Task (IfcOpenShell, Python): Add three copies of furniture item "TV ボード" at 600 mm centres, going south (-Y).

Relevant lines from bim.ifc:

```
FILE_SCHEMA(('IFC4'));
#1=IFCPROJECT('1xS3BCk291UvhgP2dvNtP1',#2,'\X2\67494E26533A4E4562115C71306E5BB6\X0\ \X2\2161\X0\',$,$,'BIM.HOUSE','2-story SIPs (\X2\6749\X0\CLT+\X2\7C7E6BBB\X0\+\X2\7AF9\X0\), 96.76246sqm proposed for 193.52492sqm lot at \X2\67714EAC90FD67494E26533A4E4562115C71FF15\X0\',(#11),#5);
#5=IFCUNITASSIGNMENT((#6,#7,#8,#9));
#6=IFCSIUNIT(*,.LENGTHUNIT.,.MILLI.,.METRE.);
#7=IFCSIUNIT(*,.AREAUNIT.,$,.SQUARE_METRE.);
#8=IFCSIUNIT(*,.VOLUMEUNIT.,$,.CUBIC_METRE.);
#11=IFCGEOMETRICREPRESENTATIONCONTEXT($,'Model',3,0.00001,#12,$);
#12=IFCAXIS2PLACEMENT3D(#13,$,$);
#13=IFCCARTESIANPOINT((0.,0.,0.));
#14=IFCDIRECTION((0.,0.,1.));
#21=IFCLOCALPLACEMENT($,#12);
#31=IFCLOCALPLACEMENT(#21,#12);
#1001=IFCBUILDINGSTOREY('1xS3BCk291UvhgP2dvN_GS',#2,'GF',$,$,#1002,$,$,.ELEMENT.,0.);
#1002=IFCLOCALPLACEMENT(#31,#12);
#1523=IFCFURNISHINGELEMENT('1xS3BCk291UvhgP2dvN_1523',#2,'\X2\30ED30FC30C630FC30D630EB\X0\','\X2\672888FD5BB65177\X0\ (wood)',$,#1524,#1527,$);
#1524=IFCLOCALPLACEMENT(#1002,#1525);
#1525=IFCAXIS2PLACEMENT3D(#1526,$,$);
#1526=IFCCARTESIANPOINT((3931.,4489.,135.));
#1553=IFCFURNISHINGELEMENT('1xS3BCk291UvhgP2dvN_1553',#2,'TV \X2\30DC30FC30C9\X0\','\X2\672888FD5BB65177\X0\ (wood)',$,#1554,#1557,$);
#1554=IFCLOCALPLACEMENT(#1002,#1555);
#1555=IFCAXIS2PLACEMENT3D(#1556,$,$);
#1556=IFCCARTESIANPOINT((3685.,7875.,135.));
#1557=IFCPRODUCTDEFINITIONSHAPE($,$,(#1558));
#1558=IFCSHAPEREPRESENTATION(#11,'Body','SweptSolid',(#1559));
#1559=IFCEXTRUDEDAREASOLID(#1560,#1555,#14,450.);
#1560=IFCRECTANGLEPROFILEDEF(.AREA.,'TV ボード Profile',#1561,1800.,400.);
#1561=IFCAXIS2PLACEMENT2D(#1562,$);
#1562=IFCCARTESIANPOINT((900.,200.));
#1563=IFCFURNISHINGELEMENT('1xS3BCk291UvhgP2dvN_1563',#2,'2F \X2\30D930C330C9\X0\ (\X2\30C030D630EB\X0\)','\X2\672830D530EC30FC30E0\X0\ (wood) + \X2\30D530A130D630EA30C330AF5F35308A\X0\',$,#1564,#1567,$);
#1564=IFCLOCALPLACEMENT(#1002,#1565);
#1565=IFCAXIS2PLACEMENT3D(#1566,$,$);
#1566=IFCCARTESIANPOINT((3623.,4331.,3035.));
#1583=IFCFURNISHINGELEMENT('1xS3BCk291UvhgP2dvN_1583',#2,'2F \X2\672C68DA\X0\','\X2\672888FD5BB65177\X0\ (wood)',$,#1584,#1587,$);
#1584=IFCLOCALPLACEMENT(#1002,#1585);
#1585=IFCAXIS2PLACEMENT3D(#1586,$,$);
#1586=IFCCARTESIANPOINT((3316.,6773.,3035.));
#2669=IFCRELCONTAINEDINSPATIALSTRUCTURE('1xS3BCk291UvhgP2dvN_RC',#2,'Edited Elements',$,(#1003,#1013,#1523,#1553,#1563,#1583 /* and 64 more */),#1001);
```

```python
import numpy as np
import ifcopenshell
import ifcopenshell.api.geometry
import ifcopenshell.api.root
import ifcopenshell.util.element
import ifcopenshell.util.placement
import ifcopenshell.util.unit

model = ifcopenshell.open("bim.ifc")
unit_scale = ifcopenshell.util.unit.calculate_unit_scale(model)


def reuse_history(source, copy):
    """copy_class also copies each property set's owner history, people and application; keep the originals."""
    for rel in copy.IsDefinedBy:
        if rel.is_a("IfcRelDefinesByProperties") and (history := rel.RelatingPropertyDefinition.OwnerHistory):
            rel.RelatingPropertyDefinition.OwnerHistory = source.OwnerHistory
            ifcopenshell.util.element.remove_deep2(model, history)


source = model.by_guid("1xS3BCk291UvhgP2dvN_1553")
base = ifcopenshell.util.placement.get_local_placement(source.ObjectPlacement)
step = np.array([0.0, -1.0, 0.0]) * 0.6 / unit_scale

for i in range(1, 4):
    copy = ifcopenshell.api.root.copy_class(model, product=source)
    copy.Representation = ifcopenshell.util.element.copy_deep(
        model, source.Representation, exclude=["IfcGeometricRepresentationContext", "IfcRepresentationMap"]
    )
    reuse_history(source, copy)
    matrix = base.copy()
    matrix[:3, 3] += i * step
    print("added at", matrix[:3, 3].round(3) + 0.0)
    ifcopenshell.api.geometry.edit_object_placement(model, product=copy, matrix=matrix, is_si=False)

model.write("bim_v2.ifc")
```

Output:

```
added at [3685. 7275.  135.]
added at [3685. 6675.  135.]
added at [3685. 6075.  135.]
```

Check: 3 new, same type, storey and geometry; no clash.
